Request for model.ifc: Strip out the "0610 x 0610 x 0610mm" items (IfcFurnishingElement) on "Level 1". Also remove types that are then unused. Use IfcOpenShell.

First a look at what the model holds.

```python
import ifcopenshell
import ifcopenshell.util.element

model = ifcopenshell.open("model.ifc")
print(model.schema)
storey = next(s for s in model.by_type("IfcBuildingStorey") if s.Name == "Level 1")
furniture = [e for e in ifcopenshell.util.element.get_decomposition(storey) if e.is_a("IfcFurnishingElement")]
seen = {}
for e in furniture:
    element_type = ifcopenshell.util.element.get_type(e)
    name = element_type.Name if element_type not in (None, e) else None
    seen[name] = seen.get(name, 0) + 1
for name, count in sorted(seen.items(), key=str):
    print(count, "x", name)
```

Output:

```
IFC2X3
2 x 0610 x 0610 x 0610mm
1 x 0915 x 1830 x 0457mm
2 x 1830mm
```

```python
import ifcopenshell
import ifcopenshell.api.root
import ifcopenshell.util.element

model = ifcopenshell.open("model.ifc")

storey = next(s for s in model.by_type("IfcBuildingStorey") if s.Name == "Level 1")
furniture = [e for e in ifcopenshell.util.element.get_decomposition(storey) if e.is_a("IfcFurnishingElement")]
targets = [e for e in furniture if (t := ifcopenshell.util.element.get_type(e)) not in (None, e) and t.Name == "0610 x 0610 x 0610mm"]
types = {ifcopenshell.util.element.get_type(e) for e in targets} - {None, *targets}

for e in targets:
    ifcopenshell.api.root.remove_product(model, product=e)
print(len(targets), "removed")

unused = [t for t in types if not ifcopenshell.util.element.get_types(t)]
for t in unused:
    ifcopenshell.api.root.remove_product(model, product=t)
print(len(unused), "unused types removed")

model.write("model_rev.ifc")
```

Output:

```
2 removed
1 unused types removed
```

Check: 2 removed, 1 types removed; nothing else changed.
